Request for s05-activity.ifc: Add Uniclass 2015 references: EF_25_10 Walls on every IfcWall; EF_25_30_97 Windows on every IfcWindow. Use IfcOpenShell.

First a look at what the model holds.

```python
import ifcopenshell

model = ifcopenshell.open("s05-activity.ifc")
print(model.schema)
print("classifications:", [c.Name for c in model.by_type("IfcClassification")])
for ifc_class in ("IfcDoor", "IfcRoof", "IfcStair", "IfcWall", "IfcWindow"):
    print(ifc_class, len(model.by_type(ifc_class)))
```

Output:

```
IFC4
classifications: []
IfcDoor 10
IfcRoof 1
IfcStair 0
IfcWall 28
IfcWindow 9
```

```python
import ifcopenshell
import ifcopenshell.api.classification

model = ifcopenshell.open("s05-activity.ifc")

system = ifcopenshell.api.classification.add_classification(model, classification="Uniclass 2015")

codes = {
    "IfcWall": ("EF_25_10", "Walls"),
    "IfcWindow": ("EF_25_30_97", "Windows"),
}
for ifc_class, (code, name) in codes.items():
    products = model.by_type(ifc_class)
    ifcopenshell.api.classification.add_reference(
        model, products=products, classification=system, identification=code, name=name
    )
    print(code, len(products))

model.write("s05-activity_rev.ifc")
```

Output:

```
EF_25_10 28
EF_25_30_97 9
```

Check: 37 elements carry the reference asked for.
